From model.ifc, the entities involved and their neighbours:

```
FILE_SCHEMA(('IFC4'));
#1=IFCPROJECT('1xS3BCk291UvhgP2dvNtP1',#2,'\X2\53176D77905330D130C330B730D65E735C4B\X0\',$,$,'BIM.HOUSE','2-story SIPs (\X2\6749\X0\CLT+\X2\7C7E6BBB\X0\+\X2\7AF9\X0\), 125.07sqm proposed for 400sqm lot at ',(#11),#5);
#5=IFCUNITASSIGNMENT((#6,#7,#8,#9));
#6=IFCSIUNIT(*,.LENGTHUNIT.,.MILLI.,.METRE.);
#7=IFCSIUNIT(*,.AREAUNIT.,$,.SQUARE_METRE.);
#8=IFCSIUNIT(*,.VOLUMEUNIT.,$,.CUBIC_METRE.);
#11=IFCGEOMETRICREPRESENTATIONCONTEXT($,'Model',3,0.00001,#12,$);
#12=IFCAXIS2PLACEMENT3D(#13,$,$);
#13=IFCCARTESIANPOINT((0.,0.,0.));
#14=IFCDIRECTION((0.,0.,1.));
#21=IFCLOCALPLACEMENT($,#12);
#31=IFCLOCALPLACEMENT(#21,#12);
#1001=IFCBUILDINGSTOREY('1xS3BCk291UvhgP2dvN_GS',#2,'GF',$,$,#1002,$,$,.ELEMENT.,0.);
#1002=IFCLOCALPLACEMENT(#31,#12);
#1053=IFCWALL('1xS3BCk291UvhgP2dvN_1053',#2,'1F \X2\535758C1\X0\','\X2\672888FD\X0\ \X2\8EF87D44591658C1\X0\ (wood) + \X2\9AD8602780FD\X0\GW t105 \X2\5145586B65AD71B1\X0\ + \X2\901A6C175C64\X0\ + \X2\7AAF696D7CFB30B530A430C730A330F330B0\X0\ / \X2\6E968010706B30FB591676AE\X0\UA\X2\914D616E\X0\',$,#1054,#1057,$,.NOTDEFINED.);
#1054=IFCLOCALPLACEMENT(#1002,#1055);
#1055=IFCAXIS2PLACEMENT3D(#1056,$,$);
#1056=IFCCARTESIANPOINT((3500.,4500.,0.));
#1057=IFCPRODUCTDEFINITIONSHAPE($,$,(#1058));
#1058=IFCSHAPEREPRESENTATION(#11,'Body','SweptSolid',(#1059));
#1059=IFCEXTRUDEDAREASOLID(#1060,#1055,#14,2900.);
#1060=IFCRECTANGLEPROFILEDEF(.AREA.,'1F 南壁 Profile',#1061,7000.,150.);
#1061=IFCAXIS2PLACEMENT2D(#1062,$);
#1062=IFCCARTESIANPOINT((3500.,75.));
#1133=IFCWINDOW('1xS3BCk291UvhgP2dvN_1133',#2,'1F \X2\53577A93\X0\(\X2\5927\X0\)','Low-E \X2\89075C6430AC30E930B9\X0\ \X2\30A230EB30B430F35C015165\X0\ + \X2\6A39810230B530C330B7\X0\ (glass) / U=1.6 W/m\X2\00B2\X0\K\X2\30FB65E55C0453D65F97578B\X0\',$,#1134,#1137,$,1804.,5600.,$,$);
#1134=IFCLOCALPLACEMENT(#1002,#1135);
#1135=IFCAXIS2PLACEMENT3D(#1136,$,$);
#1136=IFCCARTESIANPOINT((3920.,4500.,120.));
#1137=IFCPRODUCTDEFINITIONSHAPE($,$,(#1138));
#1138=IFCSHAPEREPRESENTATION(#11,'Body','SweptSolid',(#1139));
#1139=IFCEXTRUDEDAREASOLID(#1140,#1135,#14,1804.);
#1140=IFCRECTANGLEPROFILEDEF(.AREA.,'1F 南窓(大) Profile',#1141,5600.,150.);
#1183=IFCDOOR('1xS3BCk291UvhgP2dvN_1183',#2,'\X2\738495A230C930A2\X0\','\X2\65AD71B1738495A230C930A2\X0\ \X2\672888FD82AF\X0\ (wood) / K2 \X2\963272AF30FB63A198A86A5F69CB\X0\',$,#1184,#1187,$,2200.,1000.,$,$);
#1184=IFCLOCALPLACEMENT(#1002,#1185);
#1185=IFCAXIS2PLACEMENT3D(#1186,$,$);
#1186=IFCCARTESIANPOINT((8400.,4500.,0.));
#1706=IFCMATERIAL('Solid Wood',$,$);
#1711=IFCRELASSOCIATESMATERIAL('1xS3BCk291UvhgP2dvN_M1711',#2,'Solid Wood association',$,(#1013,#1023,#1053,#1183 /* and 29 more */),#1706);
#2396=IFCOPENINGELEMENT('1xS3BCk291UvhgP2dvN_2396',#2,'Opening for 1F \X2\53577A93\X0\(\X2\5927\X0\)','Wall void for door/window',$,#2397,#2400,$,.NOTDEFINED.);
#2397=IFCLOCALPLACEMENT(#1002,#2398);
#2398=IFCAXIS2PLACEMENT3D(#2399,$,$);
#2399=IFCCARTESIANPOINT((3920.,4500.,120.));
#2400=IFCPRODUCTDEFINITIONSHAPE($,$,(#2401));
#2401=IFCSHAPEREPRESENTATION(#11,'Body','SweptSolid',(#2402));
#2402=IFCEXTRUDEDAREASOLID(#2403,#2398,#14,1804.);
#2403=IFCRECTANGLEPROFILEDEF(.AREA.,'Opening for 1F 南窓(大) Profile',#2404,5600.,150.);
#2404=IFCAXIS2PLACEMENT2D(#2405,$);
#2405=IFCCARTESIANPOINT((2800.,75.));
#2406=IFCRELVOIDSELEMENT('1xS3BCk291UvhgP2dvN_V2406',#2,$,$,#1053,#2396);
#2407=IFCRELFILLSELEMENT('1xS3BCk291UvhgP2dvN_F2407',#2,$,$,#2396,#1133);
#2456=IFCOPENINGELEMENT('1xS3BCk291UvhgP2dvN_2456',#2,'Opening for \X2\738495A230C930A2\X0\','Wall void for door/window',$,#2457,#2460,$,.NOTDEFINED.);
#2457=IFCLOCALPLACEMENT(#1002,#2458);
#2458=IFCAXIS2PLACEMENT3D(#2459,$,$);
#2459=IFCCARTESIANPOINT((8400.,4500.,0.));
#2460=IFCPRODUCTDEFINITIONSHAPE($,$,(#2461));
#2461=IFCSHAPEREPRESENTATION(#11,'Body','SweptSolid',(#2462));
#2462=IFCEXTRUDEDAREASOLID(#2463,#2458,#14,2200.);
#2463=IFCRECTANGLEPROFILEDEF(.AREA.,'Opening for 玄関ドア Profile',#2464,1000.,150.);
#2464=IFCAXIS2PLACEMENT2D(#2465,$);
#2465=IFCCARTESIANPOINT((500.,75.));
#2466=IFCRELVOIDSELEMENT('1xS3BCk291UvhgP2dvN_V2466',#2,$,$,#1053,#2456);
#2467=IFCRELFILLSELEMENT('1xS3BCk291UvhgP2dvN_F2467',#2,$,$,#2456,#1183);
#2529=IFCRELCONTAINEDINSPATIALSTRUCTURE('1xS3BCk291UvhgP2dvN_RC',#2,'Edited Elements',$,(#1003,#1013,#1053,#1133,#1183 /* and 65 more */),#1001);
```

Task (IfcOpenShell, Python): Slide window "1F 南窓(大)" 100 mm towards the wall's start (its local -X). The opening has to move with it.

```python
import ifcopenshell
import ifcopenshell.api.geometry
import ifcopenshell.util.placement

model = ifcopenshell.open("model.ifc")

window = model.by_id(1133)
opening = window.FillsVoids[0].RelatingOpeningElement
wall = opening.VoidsElements[0].RelatingBuildingElement

wall_matrix = ifcopenshell.util.placement.get_local_placement(wall.ObjectPlacement)
shift = wall_matrix[:3, 0] * -100.0
before = ifcopenshell.util.placement.get_local_placement(window.ObjectPlacement)[:3, 3].copy()

# The window is not placed relative to its opening, so move both.
for product in (opening, window):
    matrix = ifcopenshell.util.placement.get_local_placement(product.ObjectPlacement)
    matrix[:3, 3] += shift
    ifcopenshell.api.geometry.edit_object_placement(model, product=product, matrix=matrix, is_si=False)

after = ifcopenshell.util.placement.get_local_placement(window.ObjectPlacement)[:3, 3]
print("window moved by", (after - before).round(3) + 0.0)

model.write("model_rev.ifc")
```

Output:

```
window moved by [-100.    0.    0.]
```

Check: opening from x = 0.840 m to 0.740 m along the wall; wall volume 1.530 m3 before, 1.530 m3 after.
